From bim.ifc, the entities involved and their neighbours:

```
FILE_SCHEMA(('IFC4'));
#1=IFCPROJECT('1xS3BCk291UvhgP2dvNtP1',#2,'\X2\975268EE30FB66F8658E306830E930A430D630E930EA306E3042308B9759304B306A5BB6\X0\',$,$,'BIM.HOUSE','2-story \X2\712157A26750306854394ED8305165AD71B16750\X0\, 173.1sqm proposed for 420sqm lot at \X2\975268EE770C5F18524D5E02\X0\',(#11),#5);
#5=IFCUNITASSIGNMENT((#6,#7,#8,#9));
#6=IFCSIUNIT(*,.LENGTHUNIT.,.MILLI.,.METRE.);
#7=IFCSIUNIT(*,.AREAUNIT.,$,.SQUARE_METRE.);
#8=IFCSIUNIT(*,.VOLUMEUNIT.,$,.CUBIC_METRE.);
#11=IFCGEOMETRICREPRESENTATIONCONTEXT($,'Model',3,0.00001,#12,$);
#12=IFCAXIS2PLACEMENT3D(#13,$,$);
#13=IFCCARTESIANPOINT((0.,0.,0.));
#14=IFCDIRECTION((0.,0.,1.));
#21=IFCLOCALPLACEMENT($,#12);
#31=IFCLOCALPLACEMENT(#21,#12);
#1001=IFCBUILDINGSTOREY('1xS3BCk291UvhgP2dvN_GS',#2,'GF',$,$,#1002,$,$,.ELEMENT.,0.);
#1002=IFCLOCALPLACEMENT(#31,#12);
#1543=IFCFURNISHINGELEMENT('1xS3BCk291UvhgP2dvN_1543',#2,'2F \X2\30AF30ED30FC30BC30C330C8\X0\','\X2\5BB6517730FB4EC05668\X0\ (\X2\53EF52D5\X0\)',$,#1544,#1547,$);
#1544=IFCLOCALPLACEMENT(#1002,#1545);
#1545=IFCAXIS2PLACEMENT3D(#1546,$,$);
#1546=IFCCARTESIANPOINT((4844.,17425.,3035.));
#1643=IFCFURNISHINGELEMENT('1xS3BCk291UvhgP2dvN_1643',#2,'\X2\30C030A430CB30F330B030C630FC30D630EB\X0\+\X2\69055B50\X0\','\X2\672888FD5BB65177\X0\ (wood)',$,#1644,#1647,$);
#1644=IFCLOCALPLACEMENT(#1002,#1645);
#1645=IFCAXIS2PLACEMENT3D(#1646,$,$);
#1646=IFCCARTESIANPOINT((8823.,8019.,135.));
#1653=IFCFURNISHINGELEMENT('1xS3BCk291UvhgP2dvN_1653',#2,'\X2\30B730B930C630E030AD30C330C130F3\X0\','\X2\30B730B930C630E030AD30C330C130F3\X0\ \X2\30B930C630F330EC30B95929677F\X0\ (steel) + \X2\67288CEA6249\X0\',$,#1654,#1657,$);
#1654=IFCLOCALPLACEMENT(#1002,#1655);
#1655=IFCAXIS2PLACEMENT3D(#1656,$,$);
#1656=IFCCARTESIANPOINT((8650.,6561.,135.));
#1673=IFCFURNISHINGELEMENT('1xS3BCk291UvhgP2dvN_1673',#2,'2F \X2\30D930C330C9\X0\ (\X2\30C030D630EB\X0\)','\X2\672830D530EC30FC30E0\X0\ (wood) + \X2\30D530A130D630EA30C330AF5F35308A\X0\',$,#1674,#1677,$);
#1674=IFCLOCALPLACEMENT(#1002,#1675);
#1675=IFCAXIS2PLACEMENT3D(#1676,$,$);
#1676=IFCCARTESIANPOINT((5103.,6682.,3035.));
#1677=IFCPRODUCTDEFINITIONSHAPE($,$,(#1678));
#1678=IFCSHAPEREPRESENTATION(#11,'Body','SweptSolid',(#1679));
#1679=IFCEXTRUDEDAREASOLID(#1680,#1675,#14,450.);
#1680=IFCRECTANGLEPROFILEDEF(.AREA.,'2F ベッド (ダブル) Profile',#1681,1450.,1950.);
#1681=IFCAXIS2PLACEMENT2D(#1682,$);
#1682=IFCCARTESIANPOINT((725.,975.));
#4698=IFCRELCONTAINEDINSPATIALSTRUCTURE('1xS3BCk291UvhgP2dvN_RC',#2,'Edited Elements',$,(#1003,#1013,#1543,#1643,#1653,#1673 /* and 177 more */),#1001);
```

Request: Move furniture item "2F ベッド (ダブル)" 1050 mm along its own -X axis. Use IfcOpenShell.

```python
import ifcopenshell
import ifcopenshell.api.geometry
import ifcopenshell.util.placement
import ifcopenshell.util.unit

model = ifcopenshell.open("bim.ifc")
unit_scale = ifcopenshell.util.unit.calculate_unit_scale(model)

item = model.by_guid("1xS3BCk291UvhgP2dvN_1673")
matrix = ifcopenshell.util.placement.get_local_placement(item.ObjectPlacement)
matrix[:3, 3] -= matrix[:3, 0] * 1.05 / unit_scale
ifcopenshell.api.geometry.edit_object_placement(model, product=item, matrix=matrix, is_si=False)

print(ifcopenshell.util.placement.get_local_placement(item.ObjectPlacement).round(3) + 0.0)

model.write("bim_edited.ifc")
```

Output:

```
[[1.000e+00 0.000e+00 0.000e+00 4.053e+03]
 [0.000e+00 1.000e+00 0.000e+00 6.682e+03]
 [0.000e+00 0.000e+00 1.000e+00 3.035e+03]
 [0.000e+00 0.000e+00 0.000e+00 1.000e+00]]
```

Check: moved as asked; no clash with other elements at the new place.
